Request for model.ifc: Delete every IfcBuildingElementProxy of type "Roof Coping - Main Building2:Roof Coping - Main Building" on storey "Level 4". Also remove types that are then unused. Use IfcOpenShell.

First a look at what the model holds.

```python
import ifcopenshell
import ifcopenshell.util.element

model = ifcopenshell.open("model.ifc")
print(model.schema)
storey = next(s for s in model.by_type("IfcBuildingStorey") if s.Name == "Level 4")
proxies = [e for e in ifcopenshell.util.element.get_decomposition(storey) if e.is_a("IfcBuildingElementProxy")]
seen = {}
for e in proxies:
    element_type = ifcopenshell.util.element.get_type(e)
    name = element_type.Name if element_type not in (None, e) else None
    seen[name] = seen.get(name, 0) + 1
for name, count in sorted(seen.items(), key=str):
    print(count, "x", name)
```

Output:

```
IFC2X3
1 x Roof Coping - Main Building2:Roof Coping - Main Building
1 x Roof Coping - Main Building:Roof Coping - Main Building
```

```python
import ifcopenshell
import ifcopenshell.api.root
import ifcopenshell.util.element

model = ifcopenshell.open("model.ifc")

storey = next(s for s in model.by_type("IfcBuildingStorey") if s.Name == "Level 4")
proxies = [e for e in ifcopenshell.util.element.get_decomposition(storey) if e.is_a("IfcBuildingElementProxy")]
targets = [e for e in proxies if (t := ifcopenshell.util.element.get_type(e)) not in (None, e) and t.Name == "Roof Coping - Main Building2:Roof Coping - Main Building"]
types = {ifcopenshell.util.element.get_type(e) for e in targets} - {None, *targets}

for e in targets:
    ifcopenshell.api.root.remove_product(model, product=e)
print(len(targets), "removed")

unused = [t for t in types if not ifcopenshell.util.element.get_types(t)]
for t in unused:
    ifcopenshell.api.root.remove_product(model, product=t)
print(len(unused), "unused types removed")

model.write("model_updated.ifc")
```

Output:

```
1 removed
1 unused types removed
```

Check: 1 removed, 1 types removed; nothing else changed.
